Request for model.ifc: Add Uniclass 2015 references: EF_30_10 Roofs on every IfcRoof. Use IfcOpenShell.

First a look at what the model holds.

```python
import ifcopenshell

model = ifcopenshell.open("model.ifc")
print(model.schema)
print("classifications:", [c.Name for c in model.by_type("IfcClassification")])
for ifc_class in ("IfcDoor", "IfcRoof", "IfcStair", "IfcWall", "IfcWindow"):
    print(ifc_class, len(model.by_type(ifc_class)))
```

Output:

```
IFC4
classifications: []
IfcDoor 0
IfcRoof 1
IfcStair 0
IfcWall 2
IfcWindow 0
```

```python
import ifcopenshell
import ifcopenshell.api.classification

model = ifcopenshell.open("model.ifc")

system = ifcopenshell.api.classification.add_classification(model, classification="Uniclass 2015")

codes = {
    "IfcRoof": ("EF_30_10", "Roofs"),
}
for ifc_class, (code, name) in codes.items():
    products = model.by_type(ifc_class)
    ifcopenshell.api.classification.add_reference(
        model, products=products, classification=system, identification=code, name=name
    )
    print(code, len(products))

model.write("model_v2.ifc")
```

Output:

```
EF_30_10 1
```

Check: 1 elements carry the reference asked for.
